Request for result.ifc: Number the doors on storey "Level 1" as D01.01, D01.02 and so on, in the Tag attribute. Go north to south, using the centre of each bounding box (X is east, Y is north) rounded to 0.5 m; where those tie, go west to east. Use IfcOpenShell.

First a look at what the model holds.

```python
import ifcopenshell
import ifcopenshell.util.element
import ifcopenshell.util.placement

model = ifcopenshell.open("result.ifc")
print(model.schema)
storey = next(s for s in model.by_type("IfcBuildingStorey") if s.Name == "Level 1")
doors = [e for e in ifcopenshell.util.element.get_decomposition(storey) if e.is_a("IfcDoor")]
for e in sorted(doors, key=lambda e: e.id()):
    origin = ifcopenshell.util.placement.get_local_placement(e.ObjectPlacement)[:3, 3]
    print(e.id(), e.Tag, e.Name, origin.round(2) + 0.0, sep=" | ")
```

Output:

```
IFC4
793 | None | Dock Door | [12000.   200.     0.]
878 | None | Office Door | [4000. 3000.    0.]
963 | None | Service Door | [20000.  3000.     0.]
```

```python
import ifcopenshell
import ifcopenshell.geom
import ifcopenshell.util.element
import ifcopenshell.util.shape

model = ifcopenshell.open("result.ifc")
settings = ifcopenshell.geom.settings()
settings.set("use-world-coords", True)


def centre(element):
    shape = ifcopenshell.geom.create_shape(settings, element)
    return ifcopenshell.util.shape.get_bbox_centroid(shape.geometry)


storey = next(s for s in model.by_type("IfcBuildingStorey") if s.Name == "Level 1")
doors = [e for e in ifcopenshell.util.element.get_decomposition(storey) if e.is_a("IfcDoor")]

# Insertion points can sit at a corner or the storey origin, so sort by the geometry (in metres).
centres = {e: centre(e) for e in doors}
doors.sort(key=lambda e: (-round(centres[e][1] / 0.5), centres[e][0]))

for i, e in enumerate(doors, start=1):
    number = f"D01.{i:02d}"
    e.Tag = number
    print(e.id(), number)

model.write("result-out.ifc")
```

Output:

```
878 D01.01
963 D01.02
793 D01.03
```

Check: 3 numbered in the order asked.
